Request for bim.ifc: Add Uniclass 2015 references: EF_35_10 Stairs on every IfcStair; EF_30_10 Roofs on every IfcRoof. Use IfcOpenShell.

First a look at what the model holds.

```python
import ifcopenshell

model = ifcopenshell.open("bim.ifc")
print(model.schema)
print("classifications:", [c.Name for c in model.by_type("IfcClassification")])
for ifc_class in ("IfcDoor", "IfcRoof", "IfcStair", "IfcWall", "IfcWindow"):
    print(ifc_class, len(model.by_type(ifc_class)))
```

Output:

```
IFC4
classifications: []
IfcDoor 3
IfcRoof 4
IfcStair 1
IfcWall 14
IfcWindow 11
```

```python
import ifcopenshell
import ifcopenshell.api.classification

model = ifcopenshell.open("bim.ifc")

system = ifcopenshell.api.classification.add_classification(model, classification="Uniclass 2015")

codes = {
    "IfcStair": ("EF_35_10", "Stairs"),
    "IfcRoof": ("EF_30_10", "Roofs"),
}
for ifc_class, (code, name) in codes.items():
    products = model.by_type(ifc_class)
    ifcopenshell.api.classification.add_reference(
        model, products=products, classification=system, identification=code, name=name
    )
    print(code, len(products))

model.write("bim_rev.ifc")
```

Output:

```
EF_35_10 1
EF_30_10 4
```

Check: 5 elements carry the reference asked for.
